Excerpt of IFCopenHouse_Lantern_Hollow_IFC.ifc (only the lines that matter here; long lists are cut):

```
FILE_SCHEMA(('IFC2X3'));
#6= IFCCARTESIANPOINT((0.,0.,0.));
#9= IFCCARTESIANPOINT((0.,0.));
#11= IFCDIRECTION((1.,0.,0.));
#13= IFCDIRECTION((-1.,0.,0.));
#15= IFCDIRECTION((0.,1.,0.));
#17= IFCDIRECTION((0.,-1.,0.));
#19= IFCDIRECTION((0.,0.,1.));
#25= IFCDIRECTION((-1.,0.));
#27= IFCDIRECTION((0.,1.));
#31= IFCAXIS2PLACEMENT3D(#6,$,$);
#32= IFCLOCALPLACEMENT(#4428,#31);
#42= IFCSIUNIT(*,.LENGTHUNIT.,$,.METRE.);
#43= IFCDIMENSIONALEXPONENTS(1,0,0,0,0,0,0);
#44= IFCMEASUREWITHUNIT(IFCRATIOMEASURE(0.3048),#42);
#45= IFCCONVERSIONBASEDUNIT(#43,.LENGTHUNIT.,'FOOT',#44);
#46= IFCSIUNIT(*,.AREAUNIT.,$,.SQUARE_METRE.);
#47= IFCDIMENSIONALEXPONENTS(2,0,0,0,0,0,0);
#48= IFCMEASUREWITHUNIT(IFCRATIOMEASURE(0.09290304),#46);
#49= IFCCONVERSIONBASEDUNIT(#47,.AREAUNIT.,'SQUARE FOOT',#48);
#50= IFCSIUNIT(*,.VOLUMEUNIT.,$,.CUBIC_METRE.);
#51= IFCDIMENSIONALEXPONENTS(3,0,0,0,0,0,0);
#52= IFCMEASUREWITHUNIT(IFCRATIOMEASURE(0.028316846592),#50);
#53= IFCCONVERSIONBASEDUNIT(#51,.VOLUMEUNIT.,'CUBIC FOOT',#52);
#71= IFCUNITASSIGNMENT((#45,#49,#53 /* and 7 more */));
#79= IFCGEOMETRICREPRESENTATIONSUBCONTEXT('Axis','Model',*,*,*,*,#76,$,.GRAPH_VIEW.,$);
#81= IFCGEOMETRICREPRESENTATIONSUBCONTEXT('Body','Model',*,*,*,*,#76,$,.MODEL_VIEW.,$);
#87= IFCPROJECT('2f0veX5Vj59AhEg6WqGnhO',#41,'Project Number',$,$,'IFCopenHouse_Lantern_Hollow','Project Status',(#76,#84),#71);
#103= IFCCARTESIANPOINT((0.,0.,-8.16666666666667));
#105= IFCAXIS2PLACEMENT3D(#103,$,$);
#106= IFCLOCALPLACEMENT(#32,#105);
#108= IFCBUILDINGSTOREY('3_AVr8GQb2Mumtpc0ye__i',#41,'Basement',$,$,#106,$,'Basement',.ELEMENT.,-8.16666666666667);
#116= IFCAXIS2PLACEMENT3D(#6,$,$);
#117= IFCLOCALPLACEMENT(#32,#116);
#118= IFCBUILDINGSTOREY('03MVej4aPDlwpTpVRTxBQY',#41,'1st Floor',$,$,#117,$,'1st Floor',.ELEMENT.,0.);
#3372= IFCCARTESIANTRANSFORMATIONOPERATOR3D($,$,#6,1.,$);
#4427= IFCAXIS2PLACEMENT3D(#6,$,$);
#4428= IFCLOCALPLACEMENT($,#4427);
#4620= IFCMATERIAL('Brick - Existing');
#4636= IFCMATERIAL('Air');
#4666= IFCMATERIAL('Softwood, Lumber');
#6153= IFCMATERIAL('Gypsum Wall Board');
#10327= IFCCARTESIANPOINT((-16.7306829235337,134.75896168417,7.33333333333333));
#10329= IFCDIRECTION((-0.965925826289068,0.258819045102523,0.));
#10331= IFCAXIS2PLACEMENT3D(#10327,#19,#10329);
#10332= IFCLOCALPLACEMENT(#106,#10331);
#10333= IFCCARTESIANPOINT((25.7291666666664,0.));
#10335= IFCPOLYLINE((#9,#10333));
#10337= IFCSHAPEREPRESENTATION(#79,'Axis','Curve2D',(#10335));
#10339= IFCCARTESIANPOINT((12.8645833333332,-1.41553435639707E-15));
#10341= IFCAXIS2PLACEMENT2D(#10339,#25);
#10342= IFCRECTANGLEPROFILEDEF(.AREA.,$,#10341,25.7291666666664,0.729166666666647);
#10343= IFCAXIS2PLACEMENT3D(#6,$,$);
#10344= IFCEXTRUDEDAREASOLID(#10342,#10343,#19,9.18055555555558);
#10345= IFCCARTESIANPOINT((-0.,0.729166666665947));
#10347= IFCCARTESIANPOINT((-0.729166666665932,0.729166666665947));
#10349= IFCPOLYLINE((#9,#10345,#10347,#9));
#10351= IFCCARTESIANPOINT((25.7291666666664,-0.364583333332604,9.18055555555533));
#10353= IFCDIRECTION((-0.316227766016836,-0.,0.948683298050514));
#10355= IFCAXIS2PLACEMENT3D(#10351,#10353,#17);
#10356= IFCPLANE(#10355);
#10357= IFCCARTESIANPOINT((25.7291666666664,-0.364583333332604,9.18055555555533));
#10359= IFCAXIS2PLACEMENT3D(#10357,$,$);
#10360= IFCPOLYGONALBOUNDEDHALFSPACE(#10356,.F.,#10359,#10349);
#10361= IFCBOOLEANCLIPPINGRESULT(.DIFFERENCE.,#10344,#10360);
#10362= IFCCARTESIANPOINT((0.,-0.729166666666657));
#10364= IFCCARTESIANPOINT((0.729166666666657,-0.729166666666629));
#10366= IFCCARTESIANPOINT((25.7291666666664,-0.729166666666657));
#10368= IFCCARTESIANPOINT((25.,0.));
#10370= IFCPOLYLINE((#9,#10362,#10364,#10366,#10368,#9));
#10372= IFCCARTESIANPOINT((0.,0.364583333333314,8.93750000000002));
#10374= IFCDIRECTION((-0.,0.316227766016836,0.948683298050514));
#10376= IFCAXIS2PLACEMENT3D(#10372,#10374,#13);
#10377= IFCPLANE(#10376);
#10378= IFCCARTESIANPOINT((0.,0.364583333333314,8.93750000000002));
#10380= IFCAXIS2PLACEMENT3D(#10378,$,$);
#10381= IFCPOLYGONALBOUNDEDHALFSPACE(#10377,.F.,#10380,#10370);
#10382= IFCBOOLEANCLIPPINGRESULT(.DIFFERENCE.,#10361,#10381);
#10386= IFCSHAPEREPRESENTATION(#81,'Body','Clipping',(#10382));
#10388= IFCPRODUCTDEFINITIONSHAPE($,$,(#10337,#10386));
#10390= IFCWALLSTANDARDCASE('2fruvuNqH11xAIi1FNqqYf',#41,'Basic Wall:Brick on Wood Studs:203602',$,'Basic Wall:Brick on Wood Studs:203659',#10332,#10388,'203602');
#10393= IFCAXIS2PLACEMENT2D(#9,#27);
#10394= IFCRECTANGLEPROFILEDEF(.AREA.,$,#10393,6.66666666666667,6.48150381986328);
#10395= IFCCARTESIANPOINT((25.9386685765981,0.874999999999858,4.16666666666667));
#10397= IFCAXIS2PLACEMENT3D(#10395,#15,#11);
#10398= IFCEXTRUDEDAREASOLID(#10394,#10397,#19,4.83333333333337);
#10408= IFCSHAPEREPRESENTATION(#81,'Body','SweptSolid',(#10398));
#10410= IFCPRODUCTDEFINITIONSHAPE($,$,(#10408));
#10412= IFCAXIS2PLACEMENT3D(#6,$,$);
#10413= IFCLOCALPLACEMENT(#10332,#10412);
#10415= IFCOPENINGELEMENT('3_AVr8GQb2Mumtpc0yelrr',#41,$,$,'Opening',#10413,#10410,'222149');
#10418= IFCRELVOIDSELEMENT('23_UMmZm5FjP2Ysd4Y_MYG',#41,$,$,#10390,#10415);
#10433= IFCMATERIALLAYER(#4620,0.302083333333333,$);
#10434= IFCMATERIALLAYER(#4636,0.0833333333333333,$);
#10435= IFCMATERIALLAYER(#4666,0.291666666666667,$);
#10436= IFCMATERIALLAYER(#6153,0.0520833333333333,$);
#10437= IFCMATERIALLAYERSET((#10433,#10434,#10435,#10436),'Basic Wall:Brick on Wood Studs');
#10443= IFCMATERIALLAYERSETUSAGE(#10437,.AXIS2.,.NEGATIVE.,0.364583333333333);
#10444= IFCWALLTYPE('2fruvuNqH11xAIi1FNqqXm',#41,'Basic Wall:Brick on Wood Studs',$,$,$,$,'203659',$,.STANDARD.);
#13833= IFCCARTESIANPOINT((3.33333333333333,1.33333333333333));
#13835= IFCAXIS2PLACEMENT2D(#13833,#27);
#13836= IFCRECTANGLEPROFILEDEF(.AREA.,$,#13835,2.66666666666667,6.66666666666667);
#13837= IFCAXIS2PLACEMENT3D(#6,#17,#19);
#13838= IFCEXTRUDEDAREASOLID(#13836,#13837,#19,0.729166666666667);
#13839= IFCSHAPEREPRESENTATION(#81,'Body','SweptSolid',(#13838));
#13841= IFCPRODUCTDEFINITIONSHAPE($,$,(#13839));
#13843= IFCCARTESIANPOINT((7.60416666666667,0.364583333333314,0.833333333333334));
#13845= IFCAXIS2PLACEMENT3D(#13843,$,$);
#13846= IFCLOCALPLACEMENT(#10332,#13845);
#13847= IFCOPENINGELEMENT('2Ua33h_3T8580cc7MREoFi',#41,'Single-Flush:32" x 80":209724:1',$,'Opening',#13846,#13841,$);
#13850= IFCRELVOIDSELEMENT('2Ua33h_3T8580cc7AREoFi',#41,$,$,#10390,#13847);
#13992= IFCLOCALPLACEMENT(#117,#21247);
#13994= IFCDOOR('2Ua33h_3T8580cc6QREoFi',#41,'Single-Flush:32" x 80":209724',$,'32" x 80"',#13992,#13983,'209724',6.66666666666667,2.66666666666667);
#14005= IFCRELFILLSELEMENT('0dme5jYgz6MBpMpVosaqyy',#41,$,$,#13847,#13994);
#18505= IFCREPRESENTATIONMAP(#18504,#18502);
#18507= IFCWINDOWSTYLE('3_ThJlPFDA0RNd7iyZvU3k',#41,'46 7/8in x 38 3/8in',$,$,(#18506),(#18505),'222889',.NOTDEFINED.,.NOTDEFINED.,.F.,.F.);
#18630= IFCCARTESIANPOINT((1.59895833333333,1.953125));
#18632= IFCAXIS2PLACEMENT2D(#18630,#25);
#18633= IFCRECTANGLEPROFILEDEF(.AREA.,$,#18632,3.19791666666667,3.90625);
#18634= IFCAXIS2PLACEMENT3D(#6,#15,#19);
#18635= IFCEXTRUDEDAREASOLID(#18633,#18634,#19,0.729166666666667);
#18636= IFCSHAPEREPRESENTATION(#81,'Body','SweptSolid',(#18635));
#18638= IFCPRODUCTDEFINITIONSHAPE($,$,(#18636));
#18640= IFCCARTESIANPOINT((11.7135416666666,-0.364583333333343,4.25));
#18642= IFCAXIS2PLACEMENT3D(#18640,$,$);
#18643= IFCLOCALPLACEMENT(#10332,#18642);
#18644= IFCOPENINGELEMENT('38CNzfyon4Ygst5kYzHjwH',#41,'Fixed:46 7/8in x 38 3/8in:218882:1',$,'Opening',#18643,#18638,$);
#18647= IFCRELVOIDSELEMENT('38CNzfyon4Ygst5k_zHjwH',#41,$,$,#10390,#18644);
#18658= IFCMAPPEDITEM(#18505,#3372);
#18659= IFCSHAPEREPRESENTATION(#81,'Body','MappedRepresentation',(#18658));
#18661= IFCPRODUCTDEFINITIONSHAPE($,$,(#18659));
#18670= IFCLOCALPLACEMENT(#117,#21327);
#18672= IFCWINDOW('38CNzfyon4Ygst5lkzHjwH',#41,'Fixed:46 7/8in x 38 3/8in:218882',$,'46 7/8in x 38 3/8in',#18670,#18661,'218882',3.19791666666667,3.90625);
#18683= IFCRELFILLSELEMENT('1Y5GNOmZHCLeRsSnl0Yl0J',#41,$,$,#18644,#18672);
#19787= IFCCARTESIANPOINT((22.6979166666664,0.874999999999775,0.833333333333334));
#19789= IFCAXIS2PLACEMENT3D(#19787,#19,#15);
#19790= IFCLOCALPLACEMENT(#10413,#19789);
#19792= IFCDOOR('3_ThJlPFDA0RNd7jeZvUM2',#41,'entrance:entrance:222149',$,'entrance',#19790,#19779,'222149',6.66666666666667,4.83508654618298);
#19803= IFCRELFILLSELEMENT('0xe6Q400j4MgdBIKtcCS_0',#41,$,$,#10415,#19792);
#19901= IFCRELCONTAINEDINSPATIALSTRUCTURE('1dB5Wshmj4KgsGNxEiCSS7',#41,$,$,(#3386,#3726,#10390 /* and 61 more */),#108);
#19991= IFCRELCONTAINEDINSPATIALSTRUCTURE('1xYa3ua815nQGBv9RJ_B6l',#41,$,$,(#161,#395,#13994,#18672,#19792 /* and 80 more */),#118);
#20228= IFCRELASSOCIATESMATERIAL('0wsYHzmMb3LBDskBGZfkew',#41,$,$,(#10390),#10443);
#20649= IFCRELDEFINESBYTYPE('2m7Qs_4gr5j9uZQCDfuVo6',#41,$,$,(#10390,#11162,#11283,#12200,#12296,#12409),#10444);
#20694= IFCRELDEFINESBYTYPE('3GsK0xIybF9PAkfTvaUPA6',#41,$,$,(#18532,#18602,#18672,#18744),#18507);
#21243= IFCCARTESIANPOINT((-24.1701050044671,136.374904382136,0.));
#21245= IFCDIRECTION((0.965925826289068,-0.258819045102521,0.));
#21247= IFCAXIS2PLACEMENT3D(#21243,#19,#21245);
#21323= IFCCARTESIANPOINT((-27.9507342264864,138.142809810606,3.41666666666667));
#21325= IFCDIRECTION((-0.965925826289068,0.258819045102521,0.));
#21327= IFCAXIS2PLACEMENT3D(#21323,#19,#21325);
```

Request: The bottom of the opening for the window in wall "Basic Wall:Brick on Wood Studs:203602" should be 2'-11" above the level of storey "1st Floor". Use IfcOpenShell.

```python
import numpy as np
import ifcopenshell
import ifcopenshell.api.geometry
import ifcopenshell.geom
import ifcopenshell.util.element
import ifcopenshell.util.placement
import ifcopenshell.util.shape
import ifcopenshell.util.unit

model = ifcopenshell.open("IFCopenHouse_Lantern_Hollow_IFC.ifc")
unit_scale = ifcopenshell.util.unit.calculate_unit_scale(model)

window = model.by_id(18672)
opening = window.FillsVoids[0].RelatingOpeningElement
storey = ifcopenshell.util.element.get_container(window, ifc_class="IfcBuildingStorey")
level = ifcopenshell.util.placement.get_local_placement(storey.ObjectPlacement)[2, 3]

# The opening's origin need not be at the sill, so measure its lowest point.
shape = ifcopenshell.geom.create_shape(ifcopenshell.geom.settings(), opening)
bottom = ifcopenshell.util.shape.get_shape_bottom_elevation(shape, shape.geometry) / unit_scale
dz = level + 35 * 0.0254 / unit_scale - bottom

shift = np.array([0.0, 0.0, dz])
# The window is not placed relative to its opening, so move both.
for product in (opening, window):
    matrix = ifcopenshell.util.placement.get_local_placement(product.ObjectPlacement)
    matrix[:3, 3] += shift
    ifcopenshell.api.geometry.edit_object_placement(model, product=product, matrix=matrix, is_si=False)

print(f"moved by {dz * unit_scale:+.3f} m")

model.write("IFCopenHouse_Lantern_Hollow_IFC_rev.ifc")
```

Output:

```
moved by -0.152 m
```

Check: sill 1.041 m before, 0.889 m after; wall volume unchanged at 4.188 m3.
